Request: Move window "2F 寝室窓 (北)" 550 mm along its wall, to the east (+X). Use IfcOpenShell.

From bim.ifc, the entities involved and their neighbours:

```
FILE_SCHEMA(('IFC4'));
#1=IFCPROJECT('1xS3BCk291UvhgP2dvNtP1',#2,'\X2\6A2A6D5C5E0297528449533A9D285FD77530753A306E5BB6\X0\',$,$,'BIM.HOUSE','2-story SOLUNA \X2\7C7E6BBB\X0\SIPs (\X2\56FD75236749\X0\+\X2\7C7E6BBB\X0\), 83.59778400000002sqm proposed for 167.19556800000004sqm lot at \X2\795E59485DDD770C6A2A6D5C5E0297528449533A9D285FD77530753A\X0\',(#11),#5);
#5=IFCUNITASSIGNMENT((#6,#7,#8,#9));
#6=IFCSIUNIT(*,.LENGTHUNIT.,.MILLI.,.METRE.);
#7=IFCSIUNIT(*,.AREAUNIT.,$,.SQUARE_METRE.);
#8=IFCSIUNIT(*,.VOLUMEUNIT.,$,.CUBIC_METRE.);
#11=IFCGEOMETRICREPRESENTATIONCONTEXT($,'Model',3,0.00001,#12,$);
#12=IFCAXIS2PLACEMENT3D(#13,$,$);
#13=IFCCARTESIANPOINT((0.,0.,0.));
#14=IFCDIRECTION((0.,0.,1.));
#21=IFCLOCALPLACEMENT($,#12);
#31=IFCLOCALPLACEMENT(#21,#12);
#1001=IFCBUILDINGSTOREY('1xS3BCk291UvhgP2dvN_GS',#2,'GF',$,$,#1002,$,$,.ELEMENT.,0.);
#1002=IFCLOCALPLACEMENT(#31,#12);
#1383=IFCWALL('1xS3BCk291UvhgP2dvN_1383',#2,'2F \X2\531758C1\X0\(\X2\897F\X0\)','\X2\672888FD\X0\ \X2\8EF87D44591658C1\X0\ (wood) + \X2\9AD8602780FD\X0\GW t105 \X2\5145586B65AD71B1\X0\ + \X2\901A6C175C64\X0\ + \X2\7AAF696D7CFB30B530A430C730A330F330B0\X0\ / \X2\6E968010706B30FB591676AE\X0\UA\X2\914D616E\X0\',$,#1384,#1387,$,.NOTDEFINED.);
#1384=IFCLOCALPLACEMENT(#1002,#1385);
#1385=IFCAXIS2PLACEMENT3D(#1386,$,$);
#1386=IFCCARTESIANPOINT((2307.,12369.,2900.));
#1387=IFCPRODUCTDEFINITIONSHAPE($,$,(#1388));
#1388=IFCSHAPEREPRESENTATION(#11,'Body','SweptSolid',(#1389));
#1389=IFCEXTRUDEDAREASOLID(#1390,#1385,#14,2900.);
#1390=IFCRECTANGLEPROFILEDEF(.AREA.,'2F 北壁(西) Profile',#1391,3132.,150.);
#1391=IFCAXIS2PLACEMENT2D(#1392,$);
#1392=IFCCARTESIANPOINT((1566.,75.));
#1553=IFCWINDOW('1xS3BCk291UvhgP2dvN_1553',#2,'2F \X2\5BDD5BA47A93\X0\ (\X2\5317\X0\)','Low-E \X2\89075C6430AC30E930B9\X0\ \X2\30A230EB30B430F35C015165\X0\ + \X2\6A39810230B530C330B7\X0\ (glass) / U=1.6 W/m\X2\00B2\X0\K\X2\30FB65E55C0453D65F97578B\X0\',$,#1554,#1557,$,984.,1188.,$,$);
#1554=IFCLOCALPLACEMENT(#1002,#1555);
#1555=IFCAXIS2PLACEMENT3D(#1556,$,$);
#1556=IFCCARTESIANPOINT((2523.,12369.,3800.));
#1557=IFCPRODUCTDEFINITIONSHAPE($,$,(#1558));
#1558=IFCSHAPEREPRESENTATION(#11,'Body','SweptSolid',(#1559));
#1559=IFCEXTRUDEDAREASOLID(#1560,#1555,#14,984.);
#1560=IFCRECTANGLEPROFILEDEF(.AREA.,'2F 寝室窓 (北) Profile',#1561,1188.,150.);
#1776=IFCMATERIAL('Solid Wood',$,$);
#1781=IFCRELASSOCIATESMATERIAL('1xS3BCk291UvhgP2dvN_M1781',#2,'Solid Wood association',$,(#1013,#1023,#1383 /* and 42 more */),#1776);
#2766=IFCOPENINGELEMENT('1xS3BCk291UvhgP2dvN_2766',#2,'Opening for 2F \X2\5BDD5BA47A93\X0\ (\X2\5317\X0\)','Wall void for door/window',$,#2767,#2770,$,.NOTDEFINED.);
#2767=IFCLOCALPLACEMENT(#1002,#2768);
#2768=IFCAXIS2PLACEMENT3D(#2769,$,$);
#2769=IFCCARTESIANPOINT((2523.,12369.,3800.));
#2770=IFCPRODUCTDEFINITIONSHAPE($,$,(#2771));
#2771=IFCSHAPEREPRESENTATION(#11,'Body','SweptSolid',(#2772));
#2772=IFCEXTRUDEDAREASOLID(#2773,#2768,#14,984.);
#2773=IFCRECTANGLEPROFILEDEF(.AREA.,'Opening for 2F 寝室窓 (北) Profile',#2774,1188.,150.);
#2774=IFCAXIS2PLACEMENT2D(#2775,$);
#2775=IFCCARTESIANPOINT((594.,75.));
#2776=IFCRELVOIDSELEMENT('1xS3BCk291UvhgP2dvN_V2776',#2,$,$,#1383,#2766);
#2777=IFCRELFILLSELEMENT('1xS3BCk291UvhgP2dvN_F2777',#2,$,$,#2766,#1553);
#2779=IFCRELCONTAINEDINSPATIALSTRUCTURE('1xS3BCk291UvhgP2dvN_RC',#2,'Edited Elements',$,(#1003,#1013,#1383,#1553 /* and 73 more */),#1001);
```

```python
import ifcopenshell
import ifcopenshell.api.geometry
import ifcopenshell.util.placement

model = ifcopenshell.open("bim.ifc")

window = model.by_guid("1xS3BCk291UvhgP2dvN_1553")
opening = window.FillsVoids[0].RelatingOpeningElement
wall = opening.VoidsElements[0].RelatingBuildingElement

wall_matrix = ifcopenshell.util.placement.get_local_placement(wall.ObjectPlacement)
shift = wall_matrix[:3, 0] * 550.0
before = ifcopenshell.util.placement.get_local_placement(window.ObjectPlacement)[:3, 3].copy()

# The window is not placed relative to its opening, so move both.
for product in (opening, window):
    matrix = ifcopenshell.util.placement.get_local_placement(product.ObjectPlacement)
    matrix[:3, 3] += shift
    ifcopenshell.api.geometry.edit_object_placement(model, product=product, matrix=matrix, is_si=False)

after = ifcopenshell.util.placement.get_local_placement(window.ObjectPlacement)[:3, 3]
print("window moved by", (after - before).round(3) + 0.0)

model.write("bim_updated.ifc")
```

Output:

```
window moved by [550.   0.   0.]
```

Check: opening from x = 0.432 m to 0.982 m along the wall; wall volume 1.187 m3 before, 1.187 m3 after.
